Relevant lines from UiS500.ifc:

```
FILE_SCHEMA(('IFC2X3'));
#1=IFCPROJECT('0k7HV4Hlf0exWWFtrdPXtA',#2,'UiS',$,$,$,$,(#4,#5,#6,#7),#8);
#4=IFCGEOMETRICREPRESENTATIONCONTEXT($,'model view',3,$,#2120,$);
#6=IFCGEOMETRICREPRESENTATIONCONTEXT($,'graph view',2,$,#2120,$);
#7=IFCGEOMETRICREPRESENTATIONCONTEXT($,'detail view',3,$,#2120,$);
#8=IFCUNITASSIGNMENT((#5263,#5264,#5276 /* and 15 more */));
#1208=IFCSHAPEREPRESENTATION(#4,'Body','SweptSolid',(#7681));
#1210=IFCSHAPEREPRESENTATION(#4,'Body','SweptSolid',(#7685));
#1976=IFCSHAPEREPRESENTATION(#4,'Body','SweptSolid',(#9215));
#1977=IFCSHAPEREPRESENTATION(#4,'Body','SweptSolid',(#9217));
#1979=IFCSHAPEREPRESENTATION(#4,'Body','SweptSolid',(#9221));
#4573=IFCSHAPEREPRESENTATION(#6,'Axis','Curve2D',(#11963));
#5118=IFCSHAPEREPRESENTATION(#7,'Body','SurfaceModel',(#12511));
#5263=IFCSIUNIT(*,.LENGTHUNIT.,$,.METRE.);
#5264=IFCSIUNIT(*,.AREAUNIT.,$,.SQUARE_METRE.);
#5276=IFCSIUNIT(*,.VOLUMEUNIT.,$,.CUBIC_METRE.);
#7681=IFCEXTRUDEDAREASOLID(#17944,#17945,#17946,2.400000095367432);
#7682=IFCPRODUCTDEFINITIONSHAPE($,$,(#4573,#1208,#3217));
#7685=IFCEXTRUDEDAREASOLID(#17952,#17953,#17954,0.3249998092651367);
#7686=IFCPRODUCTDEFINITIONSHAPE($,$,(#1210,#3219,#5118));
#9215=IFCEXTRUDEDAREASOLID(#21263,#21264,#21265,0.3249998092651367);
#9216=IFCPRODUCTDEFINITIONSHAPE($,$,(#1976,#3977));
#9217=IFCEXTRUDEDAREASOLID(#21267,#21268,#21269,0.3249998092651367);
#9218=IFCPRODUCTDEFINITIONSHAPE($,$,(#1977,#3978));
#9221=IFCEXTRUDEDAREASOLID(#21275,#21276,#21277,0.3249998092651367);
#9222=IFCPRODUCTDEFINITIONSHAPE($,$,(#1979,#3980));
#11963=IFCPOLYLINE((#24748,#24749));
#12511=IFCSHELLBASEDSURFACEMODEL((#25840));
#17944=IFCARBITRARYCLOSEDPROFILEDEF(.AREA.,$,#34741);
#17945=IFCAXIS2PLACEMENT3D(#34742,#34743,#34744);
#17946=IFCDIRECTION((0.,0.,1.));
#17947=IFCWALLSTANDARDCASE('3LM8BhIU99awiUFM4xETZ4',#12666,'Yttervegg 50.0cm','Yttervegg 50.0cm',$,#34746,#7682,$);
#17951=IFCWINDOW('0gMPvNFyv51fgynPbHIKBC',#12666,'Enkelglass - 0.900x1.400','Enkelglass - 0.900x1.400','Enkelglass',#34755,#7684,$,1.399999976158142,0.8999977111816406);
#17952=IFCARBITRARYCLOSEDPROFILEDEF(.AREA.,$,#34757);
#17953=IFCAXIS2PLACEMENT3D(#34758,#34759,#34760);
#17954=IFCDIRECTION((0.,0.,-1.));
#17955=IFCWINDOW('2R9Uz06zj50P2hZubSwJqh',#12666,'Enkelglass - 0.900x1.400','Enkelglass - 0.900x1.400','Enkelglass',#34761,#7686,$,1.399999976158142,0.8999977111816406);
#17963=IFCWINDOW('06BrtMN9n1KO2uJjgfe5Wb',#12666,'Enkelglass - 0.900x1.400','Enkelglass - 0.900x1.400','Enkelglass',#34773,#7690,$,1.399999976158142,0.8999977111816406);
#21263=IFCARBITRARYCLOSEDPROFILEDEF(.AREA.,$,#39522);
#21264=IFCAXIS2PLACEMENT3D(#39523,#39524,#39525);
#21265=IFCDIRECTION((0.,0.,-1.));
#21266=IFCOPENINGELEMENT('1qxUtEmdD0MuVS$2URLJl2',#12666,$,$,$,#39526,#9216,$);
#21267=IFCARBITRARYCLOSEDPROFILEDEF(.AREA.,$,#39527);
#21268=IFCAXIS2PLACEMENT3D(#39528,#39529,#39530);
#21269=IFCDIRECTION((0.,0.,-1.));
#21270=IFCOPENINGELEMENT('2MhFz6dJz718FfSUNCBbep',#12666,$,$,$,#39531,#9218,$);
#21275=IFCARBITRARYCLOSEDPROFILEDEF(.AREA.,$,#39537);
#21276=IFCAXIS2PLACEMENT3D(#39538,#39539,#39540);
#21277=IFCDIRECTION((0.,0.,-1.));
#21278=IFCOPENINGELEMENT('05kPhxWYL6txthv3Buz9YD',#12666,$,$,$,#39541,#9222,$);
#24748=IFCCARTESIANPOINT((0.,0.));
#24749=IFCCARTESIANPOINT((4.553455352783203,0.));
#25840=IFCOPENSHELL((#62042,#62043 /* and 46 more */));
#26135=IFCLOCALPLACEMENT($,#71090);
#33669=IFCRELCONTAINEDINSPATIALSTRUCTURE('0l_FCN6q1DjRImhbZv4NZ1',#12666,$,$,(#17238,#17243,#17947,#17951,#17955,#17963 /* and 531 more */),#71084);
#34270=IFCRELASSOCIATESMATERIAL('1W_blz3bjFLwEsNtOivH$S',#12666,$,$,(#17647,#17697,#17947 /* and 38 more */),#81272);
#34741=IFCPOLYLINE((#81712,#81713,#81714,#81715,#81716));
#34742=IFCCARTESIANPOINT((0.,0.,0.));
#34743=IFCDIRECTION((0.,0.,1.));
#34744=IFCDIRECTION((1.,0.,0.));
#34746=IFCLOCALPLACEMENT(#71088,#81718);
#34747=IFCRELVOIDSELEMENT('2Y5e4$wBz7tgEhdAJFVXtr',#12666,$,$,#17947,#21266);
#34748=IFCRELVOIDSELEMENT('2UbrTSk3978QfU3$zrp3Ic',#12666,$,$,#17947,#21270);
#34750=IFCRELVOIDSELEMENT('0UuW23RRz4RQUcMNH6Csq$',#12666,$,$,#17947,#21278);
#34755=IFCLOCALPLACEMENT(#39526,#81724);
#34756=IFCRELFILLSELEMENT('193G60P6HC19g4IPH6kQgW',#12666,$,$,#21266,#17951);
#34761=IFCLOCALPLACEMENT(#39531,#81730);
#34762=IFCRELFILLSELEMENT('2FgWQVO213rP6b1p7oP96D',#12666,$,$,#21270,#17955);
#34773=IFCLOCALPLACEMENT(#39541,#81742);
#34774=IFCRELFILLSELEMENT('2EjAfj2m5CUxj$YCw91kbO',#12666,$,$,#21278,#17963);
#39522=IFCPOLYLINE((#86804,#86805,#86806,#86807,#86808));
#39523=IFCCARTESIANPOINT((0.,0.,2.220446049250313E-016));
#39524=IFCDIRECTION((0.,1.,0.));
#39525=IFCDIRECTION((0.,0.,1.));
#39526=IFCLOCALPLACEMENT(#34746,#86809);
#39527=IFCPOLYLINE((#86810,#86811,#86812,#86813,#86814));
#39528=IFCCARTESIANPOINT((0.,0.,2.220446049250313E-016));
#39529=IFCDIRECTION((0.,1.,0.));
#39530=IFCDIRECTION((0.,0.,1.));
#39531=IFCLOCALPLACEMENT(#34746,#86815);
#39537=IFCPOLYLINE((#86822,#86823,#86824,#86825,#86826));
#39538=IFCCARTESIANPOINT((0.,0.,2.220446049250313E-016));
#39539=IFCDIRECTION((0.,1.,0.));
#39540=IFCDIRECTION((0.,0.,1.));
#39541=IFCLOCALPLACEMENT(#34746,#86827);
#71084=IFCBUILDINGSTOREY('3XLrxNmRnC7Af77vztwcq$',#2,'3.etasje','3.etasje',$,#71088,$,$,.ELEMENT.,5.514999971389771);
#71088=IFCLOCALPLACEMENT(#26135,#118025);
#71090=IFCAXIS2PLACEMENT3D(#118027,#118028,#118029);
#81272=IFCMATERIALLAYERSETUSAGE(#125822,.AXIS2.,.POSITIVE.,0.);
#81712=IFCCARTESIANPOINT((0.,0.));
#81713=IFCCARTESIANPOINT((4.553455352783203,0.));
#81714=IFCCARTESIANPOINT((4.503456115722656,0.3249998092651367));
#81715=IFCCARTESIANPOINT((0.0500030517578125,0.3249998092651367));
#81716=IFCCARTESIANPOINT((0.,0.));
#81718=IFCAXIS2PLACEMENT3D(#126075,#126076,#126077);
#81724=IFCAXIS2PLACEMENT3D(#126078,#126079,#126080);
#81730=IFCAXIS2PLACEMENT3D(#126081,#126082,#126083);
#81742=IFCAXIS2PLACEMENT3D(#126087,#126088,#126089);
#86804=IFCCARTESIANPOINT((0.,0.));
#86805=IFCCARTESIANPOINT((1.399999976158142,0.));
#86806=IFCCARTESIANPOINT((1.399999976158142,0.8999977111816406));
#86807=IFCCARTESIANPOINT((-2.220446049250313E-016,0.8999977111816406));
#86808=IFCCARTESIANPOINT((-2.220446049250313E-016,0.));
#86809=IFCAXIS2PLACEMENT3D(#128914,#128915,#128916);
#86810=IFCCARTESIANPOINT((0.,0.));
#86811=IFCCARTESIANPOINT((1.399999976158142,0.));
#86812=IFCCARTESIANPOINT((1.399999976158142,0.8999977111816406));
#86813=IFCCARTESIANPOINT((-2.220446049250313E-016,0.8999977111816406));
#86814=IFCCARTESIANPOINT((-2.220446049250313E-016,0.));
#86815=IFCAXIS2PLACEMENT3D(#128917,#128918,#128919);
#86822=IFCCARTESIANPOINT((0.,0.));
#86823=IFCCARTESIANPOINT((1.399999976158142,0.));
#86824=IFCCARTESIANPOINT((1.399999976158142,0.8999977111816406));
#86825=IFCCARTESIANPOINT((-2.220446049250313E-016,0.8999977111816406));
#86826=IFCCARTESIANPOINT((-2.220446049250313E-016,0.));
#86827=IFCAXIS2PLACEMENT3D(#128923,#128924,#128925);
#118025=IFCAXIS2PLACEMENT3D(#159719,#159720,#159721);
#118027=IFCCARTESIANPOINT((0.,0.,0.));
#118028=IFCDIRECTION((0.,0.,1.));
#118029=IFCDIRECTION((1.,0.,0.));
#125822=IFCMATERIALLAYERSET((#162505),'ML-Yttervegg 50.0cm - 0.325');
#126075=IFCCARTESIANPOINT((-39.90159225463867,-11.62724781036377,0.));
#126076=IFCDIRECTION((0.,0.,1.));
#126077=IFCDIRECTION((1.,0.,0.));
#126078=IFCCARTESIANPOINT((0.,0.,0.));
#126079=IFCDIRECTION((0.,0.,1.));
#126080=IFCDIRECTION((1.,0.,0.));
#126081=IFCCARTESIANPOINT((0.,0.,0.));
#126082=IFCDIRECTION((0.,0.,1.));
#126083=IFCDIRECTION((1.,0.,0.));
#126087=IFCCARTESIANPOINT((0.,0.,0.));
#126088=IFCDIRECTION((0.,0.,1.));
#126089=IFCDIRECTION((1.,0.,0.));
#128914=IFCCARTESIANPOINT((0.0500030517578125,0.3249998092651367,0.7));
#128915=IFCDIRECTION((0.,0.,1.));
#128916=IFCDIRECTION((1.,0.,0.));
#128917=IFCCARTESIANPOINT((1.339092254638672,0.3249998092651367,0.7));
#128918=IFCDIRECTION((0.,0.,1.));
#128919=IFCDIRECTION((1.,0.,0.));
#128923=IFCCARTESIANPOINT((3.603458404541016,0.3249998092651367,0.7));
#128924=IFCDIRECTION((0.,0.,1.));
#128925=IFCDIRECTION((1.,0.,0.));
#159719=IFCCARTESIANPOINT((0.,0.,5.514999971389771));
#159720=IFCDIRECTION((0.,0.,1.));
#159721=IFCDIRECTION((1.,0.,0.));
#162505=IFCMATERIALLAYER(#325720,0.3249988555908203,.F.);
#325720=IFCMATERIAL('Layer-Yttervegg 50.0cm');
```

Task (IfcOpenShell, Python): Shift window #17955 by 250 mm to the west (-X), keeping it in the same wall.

```python
import ifcopenshell
import ifcopenshell.api.geometry
import ifcopenshell.util.placement

model = ifcopenshell.open("UiS500.ifc")

window = model.by_guid("2R9Uz06zj50P2hZubSwJqh")
opening = window.FillsVoids[0].RelatingOpeningElement
wall = opening.VoidsElements[0].RelatingBuildingElement

wall_matrix = ifcopenshell.util.placement.get_local_placement(wall.ObjectPlacement)
shift = wall_matrix[:3, 0] * -0.25
before = ifcopenshell.util.placement.get_local_placement(window.ObjectPlacement)[:3, 3].copy()

# The window is placed relative to its opening, so it follows when the opening moves.
matrix = ifcopenshell.util.placement.get_local_placement(opening.ObjectPlacement)
matrix[:3, 3] += shift
ifcopenshell.api.geometry.edit_object_placement(
    model, product=opening, matrix=matrix, is_si=False, should_transform_children=True
)

after = ifcopenshell.util.placement.get_local_placement(window.ObjectPlacement)[:3, 3]
print("window moved by", (after - before).round(3) + 0.0)

model.write("UiS500_rev.ifc")
```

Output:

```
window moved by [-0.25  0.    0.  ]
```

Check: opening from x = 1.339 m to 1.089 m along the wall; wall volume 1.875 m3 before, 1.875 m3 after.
